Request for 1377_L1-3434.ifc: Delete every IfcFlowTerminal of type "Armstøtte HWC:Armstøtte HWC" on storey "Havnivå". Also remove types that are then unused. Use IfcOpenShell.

First a look at what the model holds.

```python
import ifcopenshell
import ifcopenshell.util.element

model = ifcopenshell.open("1377_L1-3434.ifc")
print(model.schema)
storey = next(s for s in model.by_type("IfcBuildingStorey") if s.Name == "Havnivå")
terminals = [e for e in ifcopenshell.util.element.get_decomposition(storey) if e.is_a("IfcFlowTerminal")]
seen = {}
for e in terminals:
    element_type = ifcopenshell.util.element.get_type(e)
    name = element_type.Name if element_type not in (None, e) else None
    seen[name] = seen.get(name, 0) + 1
for name, count in sorted(seen.items(), key=str):
    print(count, "x", name)
```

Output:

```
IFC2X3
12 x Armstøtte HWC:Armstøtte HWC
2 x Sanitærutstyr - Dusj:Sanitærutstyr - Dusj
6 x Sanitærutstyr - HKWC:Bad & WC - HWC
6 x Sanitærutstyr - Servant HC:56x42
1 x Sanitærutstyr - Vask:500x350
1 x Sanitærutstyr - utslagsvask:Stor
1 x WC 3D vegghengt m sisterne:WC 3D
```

```python
import ifcopenshell
import ifcopenshell.api.root
import ifcopenshell.util.element

model = ifcopenshell.open("1377_L1-3434.ifc")

storey = next(s for s in model.by_type("IfcBuildingStorey") if s.Name == "Havnivå")
terminals = [e for e in ifcopenshell.util.element.get_decomposition(storey) if e.is_a("IfcFlowTerminal")]
targets = [e for e in terminals if (t := ifcopenshell.util.element.get_type(e)) not in (None, e) and t.Name == "Armstøtte HWC:Armstøtte HWC"]
types = {ifcopenshell.util.element.get_type(e) for e in targets} - {None, *targets}

for e in targets:
    ifcopenshell.api.root.remove_product(model, product=e)
print(len(targets), "removed")

unused = [t for t in types if not ifcopenshell.util.element.get_types(t)]
for t in unused:
    ifcopenshell.api.root.remove_product(model, product=t)
print(len(unused), "unused types removed")

model.write("1377_L1-3434-out.ifc")
```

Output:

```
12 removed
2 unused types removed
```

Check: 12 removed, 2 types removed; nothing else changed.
